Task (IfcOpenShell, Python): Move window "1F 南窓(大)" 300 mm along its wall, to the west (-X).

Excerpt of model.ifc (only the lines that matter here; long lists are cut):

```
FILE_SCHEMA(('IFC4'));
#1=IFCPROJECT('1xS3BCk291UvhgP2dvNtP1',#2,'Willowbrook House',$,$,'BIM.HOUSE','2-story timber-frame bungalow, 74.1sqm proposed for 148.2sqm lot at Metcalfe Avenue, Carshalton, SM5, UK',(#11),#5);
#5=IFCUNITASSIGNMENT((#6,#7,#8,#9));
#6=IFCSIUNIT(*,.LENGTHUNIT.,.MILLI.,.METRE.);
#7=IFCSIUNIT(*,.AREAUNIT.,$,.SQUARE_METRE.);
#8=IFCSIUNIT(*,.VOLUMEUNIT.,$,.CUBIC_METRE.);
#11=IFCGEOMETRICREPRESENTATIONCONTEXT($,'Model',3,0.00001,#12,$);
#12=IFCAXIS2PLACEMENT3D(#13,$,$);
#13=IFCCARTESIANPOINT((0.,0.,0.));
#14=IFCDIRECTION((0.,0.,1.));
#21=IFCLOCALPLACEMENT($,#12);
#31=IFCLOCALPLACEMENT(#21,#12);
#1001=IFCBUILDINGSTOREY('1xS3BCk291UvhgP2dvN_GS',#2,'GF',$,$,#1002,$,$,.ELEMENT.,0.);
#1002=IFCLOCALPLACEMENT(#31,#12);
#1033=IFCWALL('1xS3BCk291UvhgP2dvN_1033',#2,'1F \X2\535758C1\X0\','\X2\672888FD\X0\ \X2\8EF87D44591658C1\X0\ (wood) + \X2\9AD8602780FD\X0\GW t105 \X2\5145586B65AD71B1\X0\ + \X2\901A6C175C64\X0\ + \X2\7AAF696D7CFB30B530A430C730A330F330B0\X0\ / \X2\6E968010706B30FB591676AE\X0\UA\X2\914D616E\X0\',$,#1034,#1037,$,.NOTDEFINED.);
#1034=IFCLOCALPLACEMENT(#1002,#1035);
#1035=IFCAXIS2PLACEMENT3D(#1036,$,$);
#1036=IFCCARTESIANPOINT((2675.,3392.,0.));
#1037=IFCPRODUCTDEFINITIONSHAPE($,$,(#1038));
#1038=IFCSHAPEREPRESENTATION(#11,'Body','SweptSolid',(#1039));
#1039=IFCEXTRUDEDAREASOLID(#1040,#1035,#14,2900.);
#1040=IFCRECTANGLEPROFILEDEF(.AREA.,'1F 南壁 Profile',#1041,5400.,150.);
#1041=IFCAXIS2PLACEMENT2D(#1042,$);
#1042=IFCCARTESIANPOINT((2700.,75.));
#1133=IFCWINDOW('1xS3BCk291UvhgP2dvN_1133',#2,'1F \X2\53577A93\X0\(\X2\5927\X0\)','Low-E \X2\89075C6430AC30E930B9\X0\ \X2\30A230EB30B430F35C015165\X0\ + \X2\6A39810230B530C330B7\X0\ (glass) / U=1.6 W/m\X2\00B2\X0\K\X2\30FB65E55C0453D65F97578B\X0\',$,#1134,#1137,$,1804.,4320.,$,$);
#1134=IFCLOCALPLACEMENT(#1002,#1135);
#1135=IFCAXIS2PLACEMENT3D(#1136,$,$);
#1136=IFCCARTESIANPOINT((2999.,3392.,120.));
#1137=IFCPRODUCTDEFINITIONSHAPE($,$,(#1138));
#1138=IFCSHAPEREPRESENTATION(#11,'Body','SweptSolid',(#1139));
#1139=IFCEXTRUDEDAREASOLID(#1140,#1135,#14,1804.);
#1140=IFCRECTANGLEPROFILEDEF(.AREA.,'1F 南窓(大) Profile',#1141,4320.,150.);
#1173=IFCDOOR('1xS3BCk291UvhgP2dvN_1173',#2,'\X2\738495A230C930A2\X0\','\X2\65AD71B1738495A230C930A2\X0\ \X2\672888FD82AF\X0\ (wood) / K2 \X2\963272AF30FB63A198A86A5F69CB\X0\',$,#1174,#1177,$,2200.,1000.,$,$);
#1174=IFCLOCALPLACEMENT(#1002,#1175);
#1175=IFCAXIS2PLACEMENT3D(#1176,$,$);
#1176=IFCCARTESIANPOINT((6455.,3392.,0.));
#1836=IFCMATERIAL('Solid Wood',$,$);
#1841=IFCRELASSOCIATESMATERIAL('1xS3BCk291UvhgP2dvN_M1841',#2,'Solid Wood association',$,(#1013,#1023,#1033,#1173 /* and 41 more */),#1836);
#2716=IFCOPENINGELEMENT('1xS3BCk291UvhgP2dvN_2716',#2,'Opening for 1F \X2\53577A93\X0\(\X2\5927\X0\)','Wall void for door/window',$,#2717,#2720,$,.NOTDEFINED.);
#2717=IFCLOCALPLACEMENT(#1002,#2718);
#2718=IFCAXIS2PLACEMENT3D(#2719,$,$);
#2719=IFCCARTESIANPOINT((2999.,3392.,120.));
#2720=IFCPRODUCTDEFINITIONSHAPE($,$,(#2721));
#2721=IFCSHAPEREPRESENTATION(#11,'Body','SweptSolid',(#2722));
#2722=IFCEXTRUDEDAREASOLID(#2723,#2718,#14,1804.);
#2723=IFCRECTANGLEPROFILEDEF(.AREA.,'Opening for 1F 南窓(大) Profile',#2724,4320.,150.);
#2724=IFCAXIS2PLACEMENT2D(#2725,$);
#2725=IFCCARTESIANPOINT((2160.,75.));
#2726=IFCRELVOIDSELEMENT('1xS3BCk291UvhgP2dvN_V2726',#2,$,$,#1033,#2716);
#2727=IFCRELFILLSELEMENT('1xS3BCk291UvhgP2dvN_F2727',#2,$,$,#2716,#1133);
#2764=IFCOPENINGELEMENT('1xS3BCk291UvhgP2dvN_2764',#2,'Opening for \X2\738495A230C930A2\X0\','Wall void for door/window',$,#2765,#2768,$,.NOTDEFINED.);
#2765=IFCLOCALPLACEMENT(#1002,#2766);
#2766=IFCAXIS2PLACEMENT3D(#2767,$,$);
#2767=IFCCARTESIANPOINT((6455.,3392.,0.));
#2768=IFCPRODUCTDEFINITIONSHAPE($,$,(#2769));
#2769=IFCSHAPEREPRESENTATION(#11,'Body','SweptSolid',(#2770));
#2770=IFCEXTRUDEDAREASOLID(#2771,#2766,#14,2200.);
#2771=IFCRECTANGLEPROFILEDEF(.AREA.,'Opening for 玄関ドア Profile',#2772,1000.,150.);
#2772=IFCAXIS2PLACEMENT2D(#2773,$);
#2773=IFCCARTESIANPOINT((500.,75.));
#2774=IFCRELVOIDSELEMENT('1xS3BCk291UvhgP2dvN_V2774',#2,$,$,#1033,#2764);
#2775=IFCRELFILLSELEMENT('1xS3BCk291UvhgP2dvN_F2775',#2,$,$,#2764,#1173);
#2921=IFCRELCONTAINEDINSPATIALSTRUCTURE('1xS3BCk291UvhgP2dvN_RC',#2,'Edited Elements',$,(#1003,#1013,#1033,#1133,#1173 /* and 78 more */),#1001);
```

```python
import ifcopenshell
import ifcopenshell.api.geometry
import ifcopenshell.util.placement
import ifcopenshell.util.unit

model = ifcopenshell.open("model.ifc")
unit_scale = ifcopenshell.util.unit.calculate_unit_scale(model)

window = model.by_guid("1xS3BCk291UvhgP2dvN_1133")
opening = window.FillsVoids[0].RelatingOpeningElement
wall = opening.VoidsElements[0].RelatingBuildingElement

wall_matrix = ifcopenshell.util.placement.get_local_placement(wall.ObjectPlacement)
shift = wall_matrix[:3, 0] * -0.3 / unit_scale
before = ifcopenshell.util.placement.get_local_placement(window.ObjectPlacement)[:3, 3].copy()

# The window is not placed relative to its opening, so move both.
for product in (opening, window):
    matrix = ifcopenshell.util.placement.get_local_placement(product.ObjectPlacement)
    matrix[:3, 3] += shift
    ifcopenshell.api.geometry.edit_object_placement(model, product=product, matrix=matrix, is_si=False)

after = ifcopenshell.util.placement.get_local_placement(window.ObjectPlacement)[:3, 3]
print("window moved by", (after - before).round(3) + 0.0)

model.write("model_edited.ifc")
```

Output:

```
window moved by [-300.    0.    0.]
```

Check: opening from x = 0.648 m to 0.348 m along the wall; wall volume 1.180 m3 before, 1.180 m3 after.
